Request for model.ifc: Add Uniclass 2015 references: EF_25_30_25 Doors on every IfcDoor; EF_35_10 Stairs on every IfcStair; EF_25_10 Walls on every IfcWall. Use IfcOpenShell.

First a look at what the model holds.

```python
import ifcopenshell

model = ifcopenshell.open("model.ifc")
print(model.schema)
print("classifications:", [c.Name for c in model.by_type("IfcClassification")])
for ifc_class in ("IfcDoor", "IfcRoof", "IfcStair", "IfcWall", "IfcWindow"):
    print(ifc_class, len(model.by_type(ifc_class)))
```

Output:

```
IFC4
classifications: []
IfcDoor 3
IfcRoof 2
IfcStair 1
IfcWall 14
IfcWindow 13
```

```python
import ifcopenshell
import ifcopenshell.api.classification

model = ifcopenshell.open("model.ifc")

system = ifcopenshell.api.classification.add_classification(model, classification="Uniclass 2015")

codes = {
    "IfcDoor": ("EF_25_30_25", "Doors"),
    "IfcStair": ("EF_35_10", "Stairs"),
    "IfcWall": ("EF_25_10", "Walls"),
}
for ifc_class, (code, name) in codes.items():
    products = model.by_type(ifc_class)
    ifcopenshell.api.classification.add_reference(
        model, products=products, classification=system, identification=code, name=name
    )
    print(code, len(products))

model.write("model-out.ifc")
```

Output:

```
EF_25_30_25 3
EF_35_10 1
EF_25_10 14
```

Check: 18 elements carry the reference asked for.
